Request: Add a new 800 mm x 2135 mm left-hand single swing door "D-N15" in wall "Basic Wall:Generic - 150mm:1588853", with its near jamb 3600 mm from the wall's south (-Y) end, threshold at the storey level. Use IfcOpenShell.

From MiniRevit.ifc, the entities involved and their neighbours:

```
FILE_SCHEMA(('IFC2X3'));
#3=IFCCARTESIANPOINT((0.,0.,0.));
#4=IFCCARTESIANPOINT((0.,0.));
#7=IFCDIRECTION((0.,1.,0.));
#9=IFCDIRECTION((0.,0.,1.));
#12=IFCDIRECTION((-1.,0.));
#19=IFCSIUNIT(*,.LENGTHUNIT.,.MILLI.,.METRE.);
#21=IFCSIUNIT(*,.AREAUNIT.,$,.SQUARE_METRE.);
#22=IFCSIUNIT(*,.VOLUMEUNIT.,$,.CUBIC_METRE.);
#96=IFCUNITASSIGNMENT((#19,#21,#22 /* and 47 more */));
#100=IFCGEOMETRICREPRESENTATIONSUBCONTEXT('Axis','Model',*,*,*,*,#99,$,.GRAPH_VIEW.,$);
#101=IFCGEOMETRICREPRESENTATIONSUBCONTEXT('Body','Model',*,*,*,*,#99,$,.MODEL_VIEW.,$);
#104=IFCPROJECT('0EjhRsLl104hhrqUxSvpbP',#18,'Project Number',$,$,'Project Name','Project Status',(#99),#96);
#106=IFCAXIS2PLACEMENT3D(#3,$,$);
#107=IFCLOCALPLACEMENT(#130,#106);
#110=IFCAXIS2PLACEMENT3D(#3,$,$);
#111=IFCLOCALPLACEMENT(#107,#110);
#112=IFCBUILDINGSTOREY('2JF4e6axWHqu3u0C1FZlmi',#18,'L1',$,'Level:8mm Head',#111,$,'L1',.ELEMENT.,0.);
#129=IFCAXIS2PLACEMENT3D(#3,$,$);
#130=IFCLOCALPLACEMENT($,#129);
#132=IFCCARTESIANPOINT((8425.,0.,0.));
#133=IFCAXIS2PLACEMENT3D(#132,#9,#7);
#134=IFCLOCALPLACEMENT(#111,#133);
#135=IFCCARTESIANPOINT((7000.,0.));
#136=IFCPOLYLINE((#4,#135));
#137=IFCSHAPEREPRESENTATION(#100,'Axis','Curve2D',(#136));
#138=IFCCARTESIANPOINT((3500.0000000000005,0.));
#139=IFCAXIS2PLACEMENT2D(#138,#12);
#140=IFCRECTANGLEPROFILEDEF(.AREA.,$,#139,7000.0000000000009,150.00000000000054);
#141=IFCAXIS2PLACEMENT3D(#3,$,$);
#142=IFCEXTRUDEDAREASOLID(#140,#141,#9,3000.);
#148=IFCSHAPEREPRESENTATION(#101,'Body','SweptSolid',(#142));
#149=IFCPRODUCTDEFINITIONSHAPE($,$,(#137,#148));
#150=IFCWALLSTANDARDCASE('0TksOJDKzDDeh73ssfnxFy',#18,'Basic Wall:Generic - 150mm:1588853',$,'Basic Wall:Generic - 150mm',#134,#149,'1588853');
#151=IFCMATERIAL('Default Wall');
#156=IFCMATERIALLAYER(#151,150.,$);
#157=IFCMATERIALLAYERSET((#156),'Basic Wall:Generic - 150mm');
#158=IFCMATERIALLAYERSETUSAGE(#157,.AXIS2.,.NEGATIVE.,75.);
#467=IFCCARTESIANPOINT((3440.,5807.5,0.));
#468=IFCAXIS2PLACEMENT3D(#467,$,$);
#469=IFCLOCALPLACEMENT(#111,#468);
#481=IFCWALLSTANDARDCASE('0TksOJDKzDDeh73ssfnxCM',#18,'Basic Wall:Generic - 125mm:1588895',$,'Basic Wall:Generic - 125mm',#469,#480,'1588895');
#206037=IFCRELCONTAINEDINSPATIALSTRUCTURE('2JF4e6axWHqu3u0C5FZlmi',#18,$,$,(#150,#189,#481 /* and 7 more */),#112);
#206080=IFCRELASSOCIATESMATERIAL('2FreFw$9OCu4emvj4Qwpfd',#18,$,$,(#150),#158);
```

```python
import numpy as np
import ifcopenshell
import ifcopenshell.api.feature
import ifcopenshell.api.geometry
import ifcopenshell.api.root
import ifcopenshell.api.spatial
import ifcopenshell.api.type
import ifcopenshell.geom
import ifcopenshell.util.element
import ifcopenshell.util.placement
import ifcopenshell.util.representation
import ifcopenshell.util.shape
import ifcopenshell.util.unit

model = ifcopenshell.open("MiniRevit.ifc")
unit_scale = ifcopenshell.util.unit.calculate_unit_scale(model)
settings = ifcopenshell.geom.settings()


def volume(element):
    """Net volume in cubic metres, openings subtracted."""
    shape = ifcopenshell.geom.create_shape(settings, element)
    return ifcopenshell.util.shape.get_volume(shape.geometry)


wall = model.by_id(150)
storey = ifcopenshell.util.element.get_container(wall, ifc_class="IfcBuildingStorey")
context = ifcopenshell.util.representation.get_context(model, "Model", "Body", "MODEL_VIEW")
before = volume(wall)

width, height, from_end, sill = 0.8, 2.135, 3.6, 0.0  # metres

# The wall runs along its own X axis, and the end named is its -X end.
wall_shape = ifcopenshell.geom.create_shape(settings, wall)
x, y, z = ifcopenshell.util.shape.get_vertices(wall_shape.geometry).T
start = x.min() + from_end
face, thickness = float(y.min()), float(y.max() - y.min())
wall_matrix = ifcopenshell.util.placement.get_local_placement(wall.ObjectPlacement)
level = ifcopenshell.util.placement.get_local_placement(storey.ObjectPlacement)[2, 3]


def in_wall(x, y):
    """Placement at x, y metres in the wall's axes, at sill height."""
    matrix = wall_matrix.copy()
    matrix[:, 3] = wall_matrix @ np.array([x / unit_scale, y / unit_scale, 0.0, 1.0])
    matrix[2, 3] = level + sill / unit_scale
    return matrix


# Opening: a box that overshoots both wall faces by 50 mm.
opening = ifcopenshell.api.root.create_entity(model, ifc_class="IfcOpeningElement")
box = ifcopenshell.api.geometry.add_wall_representation(
    model, context=context, length=width, height=height, thickness=thickness + 0.1
)
ifcopenshell.api.geometry.assign_representation(model, product=opening, representation=box)
ifcopenshell.api.geometry.edit_object_placement(model, product=opening, matrix=in_wall(start, face - 0.05), is_si=False)
ifcopenshell.api.feature.add_feature(model, feature=opening, element=wall)

door = ifcopenshell.api.root.create_entity(model, ifc_class="IfcDoor", name="D-N15")
door.OverallWidth, door.OverallHeight = width / unit_scale, height / unit_scale
body = ifcopenshell.api.geometry.add_door_representation(
    model,
    context=context,
    overall_width=door.OverallWidth,
    overall_height=door.OverallHeight,
    operation_type="SINGLE_SWING_LEFT",
    lining_properties={"LiningDepth": thickness / unit_scale, "ThresholdDepth": thickness / unit_scale},
)
ifcopenshell.api.geometry.assign_representation(model, product=door, representation=body)
ifcopenshell.api.spatial.assign_container(model, products=[door], relating_structure=storey)
fills = ifcopenshell.api.feature.add_filling(model, opening=opening, element=door)
fills.OwnerHistory = door.OwnerHistory  # required in IFC2X3

# IFC2X3 keeps the operation on the door style.
style = ifcopenshell.api.root.create_entity(model, ifc_class="IfcDoorStyle", name="D-N15")
style.OperationType, style.ConstructionType = "SINGLE_SWING_LEFT", "NOTDEFINED"
style.ParameterTakesPrecedence = style.Sizeable = False
ifcopenshell.api.type.assign_type(model, related_objects=[door], relating_type=style)

# The lining spans the wall, so the door starts at the wall face.
ifcopenshell.api.geometry.edit_object_placement(model, product=door, matrix=in_wall(start, face), is_si=False)

after = volume(wall)

print(f"wall volume {before:.3f} -> {after:.3f} m3")

model.write("MiniRevit_updated.ifc")
```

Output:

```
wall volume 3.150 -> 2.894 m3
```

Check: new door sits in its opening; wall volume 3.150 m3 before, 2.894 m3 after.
